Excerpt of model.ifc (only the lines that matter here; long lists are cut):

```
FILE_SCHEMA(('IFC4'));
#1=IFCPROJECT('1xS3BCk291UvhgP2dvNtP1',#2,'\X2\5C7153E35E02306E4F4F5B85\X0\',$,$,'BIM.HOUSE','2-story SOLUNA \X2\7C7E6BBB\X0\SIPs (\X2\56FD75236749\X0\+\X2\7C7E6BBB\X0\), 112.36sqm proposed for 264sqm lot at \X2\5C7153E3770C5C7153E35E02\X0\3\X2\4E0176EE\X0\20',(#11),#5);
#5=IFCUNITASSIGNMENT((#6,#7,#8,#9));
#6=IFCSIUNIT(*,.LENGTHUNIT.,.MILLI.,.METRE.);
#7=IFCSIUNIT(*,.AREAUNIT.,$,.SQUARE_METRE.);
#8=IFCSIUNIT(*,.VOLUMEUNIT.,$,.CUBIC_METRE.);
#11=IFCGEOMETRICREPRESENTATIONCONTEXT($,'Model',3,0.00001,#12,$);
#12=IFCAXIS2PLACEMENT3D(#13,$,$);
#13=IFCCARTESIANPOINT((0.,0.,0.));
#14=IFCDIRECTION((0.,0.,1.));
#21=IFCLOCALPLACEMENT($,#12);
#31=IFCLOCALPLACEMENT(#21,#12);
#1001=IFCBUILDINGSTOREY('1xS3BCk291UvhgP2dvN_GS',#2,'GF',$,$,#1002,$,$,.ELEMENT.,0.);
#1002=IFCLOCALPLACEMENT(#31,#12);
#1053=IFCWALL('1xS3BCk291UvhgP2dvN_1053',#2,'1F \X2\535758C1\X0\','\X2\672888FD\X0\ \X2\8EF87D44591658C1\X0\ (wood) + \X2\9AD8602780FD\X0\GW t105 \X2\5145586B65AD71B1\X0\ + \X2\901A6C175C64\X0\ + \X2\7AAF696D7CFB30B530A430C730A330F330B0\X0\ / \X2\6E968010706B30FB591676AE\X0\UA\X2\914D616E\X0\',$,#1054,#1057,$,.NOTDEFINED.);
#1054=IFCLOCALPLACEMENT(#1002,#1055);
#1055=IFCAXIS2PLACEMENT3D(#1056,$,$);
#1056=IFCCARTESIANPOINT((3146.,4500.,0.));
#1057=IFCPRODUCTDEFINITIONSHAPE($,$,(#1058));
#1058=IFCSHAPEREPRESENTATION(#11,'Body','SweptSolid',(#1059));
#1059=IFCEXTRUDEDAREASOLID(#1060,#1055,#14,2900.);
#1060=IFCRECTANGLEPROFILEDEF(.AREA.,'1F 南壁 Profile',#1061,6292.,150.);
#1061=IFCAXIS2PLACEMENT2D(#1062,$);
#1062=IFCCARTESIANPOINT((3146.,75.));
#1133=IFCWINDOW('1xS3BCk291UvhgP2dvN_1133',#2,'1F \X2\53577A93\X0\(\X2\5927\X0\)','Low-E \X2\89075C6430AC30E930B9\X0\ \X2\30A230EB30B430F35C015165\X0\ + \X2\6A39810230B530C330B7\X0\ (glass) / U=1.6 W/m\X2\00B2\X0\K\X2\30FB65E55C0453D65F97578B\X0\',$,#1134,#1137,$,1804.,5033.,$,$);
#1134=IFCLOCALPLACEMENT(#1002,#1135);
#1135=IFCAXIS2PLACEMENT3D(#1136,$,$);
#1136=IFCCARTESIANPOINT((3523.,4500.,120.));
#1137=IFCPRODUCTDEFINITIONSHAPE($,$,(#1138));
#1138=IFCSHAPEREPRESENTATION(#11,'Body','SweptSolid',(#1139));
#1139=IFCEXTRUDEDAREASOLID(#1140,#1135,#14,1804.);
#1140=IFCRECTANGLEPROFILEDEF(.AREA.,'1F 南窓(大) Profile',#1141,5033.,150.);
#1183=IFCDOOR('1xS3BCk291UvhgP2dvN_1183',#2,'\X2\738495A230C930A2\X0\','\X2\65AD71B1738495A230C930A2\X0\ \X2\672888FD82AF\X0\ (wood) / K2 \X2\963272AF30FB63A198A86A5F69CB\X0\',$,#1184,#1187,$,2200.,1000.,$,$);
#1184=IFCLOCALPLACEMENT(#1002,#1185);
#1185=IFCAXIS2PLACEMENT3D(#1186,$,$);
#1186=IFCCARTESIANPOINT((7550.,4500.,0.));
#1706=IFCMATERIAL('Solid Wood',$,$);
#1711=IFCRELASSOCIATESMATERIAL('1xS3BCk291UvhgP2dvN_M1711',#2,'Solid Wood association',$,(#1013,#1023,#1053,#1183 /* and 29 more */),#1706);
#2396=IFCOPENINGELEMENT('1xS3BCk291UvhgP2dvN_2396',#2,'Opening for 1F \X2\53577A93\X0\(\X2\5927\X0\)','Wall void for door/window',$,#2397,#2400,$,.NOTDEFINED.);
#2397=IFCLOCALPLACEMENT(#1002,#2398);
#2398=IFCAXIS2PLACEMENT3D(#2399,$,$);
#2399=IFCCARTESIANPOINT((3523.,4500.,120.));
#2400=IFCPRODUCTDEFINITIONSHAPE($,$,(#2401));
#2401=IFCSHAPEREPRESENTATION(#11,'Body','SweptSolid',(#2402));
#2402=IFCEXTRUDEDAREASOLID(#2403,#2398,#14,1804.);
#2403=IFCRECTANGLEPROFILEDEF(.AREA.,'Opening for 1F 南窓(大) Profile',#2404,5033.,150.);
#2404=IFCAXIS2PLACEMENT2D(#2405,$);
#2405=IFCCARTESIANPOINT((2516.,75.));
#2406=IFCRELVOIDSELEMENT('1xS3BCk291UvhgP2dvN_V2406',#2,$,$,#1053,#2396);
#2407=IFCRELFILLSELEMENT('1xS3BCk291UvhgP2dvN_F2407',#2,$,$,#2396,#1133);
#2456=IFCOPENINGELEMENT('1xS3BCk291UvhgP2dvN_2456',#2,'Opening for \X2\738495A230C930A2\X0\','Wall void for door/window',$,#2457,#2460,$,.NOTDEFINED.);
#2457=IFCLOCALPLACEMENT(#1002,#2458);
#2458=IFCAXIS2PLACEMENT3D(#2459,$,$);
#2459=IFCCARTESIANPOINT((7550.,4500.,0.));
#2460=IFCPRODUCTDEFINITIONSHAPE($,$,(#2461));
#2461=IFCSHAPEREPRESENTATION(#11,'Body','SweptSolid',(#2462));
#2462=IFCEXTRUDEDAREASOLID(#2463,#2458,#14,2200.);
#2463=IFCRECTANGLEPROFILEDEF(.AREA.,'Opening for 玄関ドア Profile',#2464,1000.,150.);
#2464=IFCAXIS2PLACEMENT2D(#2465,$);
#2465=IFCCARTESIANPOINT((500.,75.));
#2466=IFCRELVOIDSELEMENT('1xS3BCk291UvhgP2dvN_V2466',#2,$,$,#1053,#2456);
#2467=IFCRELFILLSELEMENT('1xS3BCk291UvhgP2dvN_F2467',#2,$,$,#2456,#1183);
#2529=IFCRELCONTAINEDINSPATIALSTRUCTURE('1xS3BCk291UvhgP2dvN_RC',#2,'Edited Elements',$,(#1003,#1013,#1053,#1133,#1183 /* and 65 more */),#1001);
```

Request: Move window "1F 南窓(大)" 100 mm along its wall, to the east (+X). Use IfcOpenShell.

```python
import ifcopenshell
import ifcopenshell.api.geometry
import ifcopenshell.util.placement

model = ifcopenshell.open("model.ifc")

window = model.by_id(1133)
opening = window.FillsVoids[0].RelatingOpeningElement
wall = opening.VoidsElements[0].RelatingBuildingElement

wall_matrix = ifcopenshell.util.placement.get_local_placement(wall.ObjectPlacement)
shift = wall_matrix[:3, 0] * 100.0
before = ifcopenshell.util.placement.get_local_placement(window.ObjectPlacement)[:3, 3].copy()

# The window is not placed relative to its opening, so move both.
for product in (opening, window):
    matrix = ifcopenshell.util.placement.get_local_placement(product.ObjectPlacement)
    matrix[:3, 3] += shift
    ifcopenshell.api.geometry.edit_object_placement(model, product=product, matrix=matrix, is_si=False)

after = ifcopenshell.util.placement.get_local_placement(window.ObjectPlacement)[:3, 3]
print("window moved by", (after - before).round(3) + 0.0)

model.write("model_v2.ifc")
```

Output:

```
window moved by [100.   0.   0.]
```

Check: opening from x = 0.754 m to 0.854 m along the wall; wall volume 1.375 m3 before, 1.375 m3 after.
